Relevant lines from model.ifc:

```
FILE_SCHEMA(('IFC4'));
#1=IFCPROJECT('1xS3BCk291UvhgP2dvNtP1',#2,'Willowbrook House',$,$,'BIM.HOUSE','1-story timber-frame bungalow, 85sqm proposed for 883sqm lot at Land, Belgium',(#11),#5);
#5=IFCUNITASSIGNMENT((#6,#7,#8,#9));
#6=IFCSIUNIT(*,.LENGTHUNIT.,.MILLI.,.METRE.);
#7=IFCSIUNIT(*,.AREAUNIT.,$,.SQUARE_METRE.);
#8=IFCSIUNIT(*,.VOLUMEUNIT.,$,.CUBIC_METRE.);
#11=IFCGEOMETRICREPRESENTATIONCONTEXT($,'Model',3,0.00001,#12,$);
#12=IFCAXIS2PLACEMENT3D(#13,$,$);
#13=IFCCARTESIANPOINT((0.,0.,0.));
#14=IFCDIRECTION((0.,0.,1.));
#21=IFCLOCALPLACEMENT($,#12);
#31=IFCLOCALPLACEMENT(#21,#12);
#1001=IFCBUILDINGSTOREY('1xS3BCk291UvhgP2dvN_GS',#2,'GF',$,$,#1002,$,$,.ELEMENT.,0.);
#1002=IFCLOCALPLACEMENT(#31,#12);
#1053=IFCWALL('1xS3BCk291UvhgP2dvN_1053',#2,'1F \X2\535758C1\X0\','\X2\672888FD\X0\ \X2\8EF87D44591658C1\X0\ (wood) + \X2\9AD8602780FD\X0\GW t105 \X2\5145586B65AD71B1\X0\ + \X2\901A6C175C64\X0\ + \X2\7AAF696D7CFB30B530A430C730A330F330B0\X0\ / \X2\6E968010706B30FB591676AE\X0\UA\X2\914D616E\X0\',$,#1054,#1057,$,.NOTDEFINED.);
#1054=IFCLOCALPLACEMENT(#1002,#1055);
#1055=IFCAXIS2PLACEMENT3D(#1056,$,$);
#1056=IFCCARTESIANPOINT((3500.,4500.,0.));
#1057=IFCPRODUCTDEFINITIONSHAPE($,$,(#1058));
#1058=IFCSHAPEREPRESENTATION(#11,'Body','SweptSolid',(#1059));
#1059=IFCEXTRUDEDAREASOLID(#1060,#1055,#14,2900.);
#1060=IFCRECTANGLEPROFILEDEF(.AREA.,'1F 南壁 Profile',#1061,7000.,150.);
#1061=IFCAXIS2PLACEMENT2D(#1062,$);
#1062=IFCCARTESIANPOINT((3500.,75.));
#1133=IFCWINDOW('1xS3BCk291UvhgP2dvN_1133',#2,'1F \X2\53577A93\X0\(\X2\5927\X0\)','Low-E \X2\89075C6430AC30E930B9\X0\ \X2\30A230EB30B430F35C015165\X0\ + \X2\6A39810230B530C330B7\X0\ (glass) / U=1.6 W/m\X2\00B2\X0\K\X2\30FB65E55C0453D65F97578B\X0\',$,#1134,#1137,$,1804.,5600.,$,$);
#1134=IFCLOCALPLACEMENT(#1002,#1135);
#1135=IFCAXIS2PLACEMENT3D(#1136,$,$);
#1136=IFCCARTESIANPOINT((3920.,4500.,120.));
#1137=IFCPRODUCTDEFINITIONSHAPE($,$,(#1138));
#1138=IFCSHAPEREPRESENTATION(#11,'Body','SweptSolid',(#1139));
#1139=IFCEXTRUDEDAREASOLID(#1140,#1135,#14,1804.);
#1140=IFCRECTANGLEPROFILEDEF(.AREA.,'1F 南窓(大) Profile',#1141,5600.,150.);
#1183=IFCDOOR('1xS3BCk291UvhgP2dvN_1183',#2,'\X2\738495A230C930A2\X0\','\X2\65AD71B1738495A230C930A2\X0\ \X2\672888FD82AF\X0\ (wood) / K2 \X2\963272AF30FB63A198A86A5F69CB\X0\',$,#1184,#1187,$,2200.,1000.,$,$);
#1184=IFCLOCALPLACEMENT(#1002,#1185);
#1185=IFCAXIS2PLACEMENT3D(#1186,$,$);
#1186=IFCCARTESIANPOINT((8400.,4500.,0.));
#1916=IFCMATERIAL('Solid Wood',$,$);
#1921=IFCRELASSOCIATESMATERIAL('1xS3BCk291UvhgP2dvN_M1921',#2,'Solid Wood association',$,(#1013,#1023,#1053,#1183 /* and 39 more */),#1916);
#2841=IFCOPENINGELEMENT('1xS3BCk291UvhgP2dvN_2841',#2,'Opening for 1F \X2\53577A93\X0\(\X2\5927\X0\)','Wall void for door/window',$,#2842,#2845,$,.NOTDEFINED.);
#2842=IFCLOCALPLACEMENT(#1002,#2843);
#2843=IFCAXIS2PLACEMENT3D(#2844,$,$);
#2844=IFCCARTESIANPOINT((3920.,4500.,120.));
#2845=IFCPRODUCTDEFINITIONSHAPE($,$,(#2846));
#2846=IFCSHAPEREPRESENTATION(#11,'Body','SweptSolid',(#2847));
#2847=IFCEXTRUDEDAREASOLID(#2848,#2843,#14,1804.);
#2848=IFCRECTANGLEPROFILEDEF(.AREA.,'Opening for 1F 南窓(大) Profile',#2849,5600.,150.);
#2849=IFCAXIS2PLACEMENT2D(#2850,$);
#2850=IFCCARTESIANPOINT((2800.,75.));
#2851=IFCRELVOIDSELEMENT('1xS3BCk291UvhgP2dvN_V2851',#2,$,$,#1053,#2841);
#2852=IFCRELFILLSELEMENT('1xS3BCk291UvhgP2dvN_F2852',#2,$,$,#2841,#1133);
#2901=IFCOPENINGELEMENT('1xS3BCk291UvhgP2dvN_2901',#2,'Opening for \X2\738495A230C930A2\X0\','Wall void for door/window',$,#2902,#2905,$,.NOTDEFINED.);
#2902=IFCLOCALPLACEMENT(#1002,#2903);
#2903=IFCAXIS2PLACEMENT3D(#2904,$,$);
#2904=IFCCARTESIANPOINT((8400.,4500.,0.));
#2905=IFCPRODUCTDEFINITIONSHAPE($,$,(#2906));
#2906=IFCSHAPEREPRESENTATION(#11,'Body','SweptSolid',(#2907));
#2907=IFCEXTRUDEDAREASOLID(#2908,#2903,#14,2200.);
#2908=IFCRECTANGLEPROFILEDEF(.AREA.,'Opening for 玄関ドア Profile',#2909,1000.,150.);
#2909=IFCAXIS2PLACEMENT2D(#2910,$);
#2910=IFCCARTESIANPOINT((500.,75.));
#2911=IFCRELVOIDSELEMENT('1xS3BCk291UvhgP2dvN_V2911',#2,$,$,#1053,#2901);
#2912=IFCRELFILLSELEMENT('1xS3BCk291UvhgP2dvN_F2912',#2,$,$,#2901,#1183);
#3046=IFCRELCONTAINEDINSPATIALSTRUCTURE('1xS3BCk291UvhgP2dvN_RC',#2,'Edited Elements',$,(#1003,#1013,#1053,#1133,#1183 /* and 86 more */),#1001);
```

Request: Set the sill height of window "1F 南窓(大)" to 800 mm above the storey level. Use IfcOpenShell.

```python
import numpy as np
import ifcopenshell
import ifcopenshell.api.geometry
import ifcopenshell.geom
import ifcopenshell.util.element
import ifcopenshell.util.placement
import ifcopenshell.util.shape
import ifcopenshell.util.unit

model = ifcopenshell.open("model.ifc")
unit_scale = ifcopenshell.util.unit.calculate_unit_scale(model)

window = model.by_id(1133)
opening = window.FillsVoids[0].RelatingOpeningElement
storey = ifcopenshell.util.element.get_container(window, ifc_class="IfcBuildingStorey")
level = ifcopenshell.util.placement.get_local_placement(storey.ObjectPlacement)[2, 3]

# The opening's origin need not be at the sill, so measure its lowest point.
shape = ifcopenshell.geom.create_shape(ifcopenshell.geom.settings(), opening)
bottom = ifcopenshell.util.shape.get_shape_bottom_elevation(shape, shape.geometry) / unit_scale
dz = level + 800.0 - bottom

shift = np.array([0.0, 0.0, dz])
# The window is not placed relative to its opening, so move both.
for product in (opening, window):
    matrix = ifcopenshell.util.placement.get_local_placement(product.ObjectPlacement)
    matrix[:3, 3] += shift
    ifcopenshell.api.geometry.edit_object_placement(model, product=product, matrix=matrix, is_si=False)

print(f"moved by {dz * unit_scale:+.3f} m")

model.write("model_v2.ifc")
```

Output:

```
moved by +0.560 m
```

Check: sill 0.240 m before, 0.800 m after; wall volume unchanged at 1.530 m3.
